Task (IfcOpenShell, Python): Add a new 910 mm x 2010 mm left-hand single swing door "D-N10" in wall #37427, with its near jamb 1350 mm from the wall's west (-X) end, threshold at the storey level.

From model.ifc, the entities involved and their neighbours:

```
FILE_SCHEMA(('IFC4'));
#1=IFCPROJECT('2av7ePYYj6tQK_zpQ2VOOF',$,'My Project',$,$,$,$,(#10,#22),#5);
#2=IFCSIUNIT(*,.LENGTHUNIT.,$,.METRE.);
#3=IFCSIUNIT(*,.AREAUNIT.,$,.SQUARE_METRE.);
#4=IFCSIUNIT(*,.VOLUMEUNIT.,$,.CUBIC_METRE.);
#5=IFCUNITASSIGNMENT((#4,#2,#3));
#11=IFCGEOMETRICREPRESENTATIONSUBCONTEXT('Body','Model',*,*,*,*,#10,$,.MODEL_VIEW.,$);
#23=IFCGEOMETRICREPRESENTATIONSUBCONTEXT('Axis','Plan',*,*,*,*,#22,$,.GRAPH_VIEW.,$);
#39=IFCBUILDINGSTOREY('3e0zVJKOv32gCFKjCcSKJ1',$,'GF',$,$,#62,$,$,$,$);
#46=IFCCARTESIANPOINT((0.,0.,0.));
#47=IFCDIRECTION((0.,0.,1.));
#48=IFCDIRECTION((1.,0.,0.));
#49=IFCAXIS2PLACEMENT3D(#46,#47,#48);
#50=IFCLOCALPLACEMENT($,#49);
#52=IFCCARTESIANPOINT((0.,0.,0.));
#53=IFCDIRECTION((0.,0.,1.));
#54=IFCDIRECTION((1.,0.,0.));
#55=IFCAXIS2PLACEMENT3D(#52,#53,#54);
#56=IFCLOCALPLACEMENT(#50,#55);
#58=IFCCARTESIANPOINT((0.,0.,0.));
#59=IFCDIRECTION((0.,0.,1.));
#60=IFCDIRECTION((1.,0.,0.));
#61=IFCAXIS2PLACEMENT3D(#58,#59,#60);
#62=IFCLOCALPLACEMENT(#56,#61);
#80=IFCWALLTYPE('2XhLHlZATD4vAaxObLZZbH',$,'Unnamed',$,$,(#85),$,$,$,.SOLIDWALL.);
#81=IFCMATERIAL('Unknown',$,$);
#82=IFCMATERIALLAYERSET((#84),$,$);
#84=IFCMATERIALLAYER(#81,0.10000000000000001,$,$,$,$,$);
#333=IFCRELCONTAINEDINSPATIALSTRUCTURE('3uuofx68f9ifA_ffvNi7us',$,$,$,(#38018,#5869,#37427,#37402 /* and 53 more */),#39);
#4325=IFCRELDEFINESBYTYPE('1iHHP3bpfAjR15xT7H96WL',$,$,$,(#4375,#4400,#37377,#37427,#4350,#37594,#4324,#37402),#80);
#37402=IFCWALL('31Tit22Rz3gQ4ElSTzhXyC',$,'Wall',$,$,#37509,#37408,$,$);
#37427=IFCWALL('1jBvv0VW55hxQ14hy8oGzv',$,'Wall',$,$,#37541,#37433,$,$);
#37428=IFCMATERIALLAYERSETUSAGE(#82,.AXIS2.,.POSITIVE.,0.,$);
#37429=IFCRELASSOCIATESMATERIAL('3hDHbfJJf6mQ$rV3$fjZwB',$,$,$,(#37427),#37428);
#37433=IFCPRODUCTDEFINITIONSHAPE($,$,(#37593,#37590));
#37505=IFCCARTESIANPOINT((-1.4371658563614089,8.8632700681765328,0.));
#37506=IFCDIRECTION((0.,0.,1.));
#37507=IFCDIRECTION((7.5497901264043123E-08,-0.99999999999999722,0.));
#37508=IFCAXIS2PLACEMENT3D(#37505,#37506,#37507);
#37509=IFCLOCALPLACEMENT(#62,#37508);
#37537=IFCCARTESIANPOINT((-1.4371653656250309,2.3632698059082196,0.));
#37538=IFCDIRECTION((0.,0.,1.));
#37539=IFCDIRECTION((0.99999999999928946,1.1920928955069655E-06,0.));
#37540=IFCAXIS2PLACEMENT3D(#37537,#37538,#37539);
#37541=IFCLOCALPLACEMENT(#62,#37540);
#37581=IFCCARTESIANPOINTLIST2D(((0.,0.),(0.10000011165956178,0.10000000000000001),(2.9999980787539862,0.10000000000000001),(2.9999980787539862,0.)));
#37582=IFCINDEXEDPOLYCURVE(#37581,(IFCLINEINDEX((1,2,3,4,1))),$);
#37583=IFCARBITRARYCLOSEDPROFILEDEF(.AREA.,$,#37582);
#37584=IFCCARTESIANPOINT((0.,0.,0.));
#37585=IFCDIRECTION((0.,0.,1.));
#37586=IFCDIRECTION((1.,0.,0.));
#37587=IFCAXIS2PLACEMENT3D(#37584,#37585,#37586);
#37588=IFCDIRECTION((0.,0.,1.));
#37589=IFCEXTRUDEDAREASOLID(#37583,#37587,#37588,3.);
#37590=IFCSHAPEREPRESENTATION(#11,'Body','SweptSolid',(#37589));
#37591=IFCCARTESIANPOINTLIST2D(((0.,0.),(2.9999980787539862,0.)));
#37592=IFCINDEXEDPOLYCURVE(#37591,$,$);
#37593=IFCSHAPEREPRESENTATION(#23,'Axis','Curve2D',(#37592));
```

```python
import numpy as np
import ifcopenshell
import ifcopenshell.api.feature
import ifcopenshell.api.geometry
import ifcopenshell.api.root
import ifcopenshell.api.spatial
import ifcopenshell.geom
import ifcopenshell.util.element
import ifcopenshell.util.placement
import ifcopenshell.util.representation
import ifcopenshell.util.shape
import ifcopenshell.util.unit

model = ifcopenshell.open("model.ifc")
unit_scale = ifcopenshell.util.unit.calculate_unit_scale(model)
settings = ifcopenshell.geom.settings()


def volume(element):
    """Net volume in cubic metres, openings subtracted."""
    shape = ifcopenshell.geom.create_shape(settings, element)
    return ifcopenshell.util.shape.get_volume(shape.geometry)


wall = model.by_guid("1jBvv0VW55hxQ14hy8oGzv")
storey = ifcopenshell.util.element.get_container(wall, ifc_class="IfcBuildingStorey")
context = ifcopenshell.util.representation.get_context(model, "Model", "Body", "MODEL_VIEW")
before = volume(wall)

width, height, from_end, sill = 0.91, 2.01, 1.35, 0.0  # metres

# The wall runs along its own X axis, and the end named is its -X end.
wall_shape = ifcopenshell.geom.create_shape(settings, wall)
x, y, z = ifcopenshell.util.shape.get_vertices(wall_shape.geometry).T
start = x.min() + from_end
face, thickness = float(y.min()), float(y.max() - y.min())
wall_matrix = ifcopenshell.util.placement.get_local_placement(wall.ObjectPlacement)
level = ifcopenshell.util.placement.get_local_placement(storey.ObjectPlacement)[2, 3]


def in_wall(x, y):
    """Placement at x, y metres in the wall's axes, at sill height."""
    matrix = wall_matrix.copy()
    matrix[:, 3] = wall_matrix @ np.array([x / unit_scale, y / unit_scale, 0.0, 1.0])
    matrix[2, 3] = level + sill / unit_scale
    return matrix


# Opening: a box that overshoots both wall faces by 50 mm.
opening = ifcopenshell.api.root.create_entity(model, ifc_class="IfcOpeningElement", predefined_type="OPENING")
box = ifcopenshell.api.geometry.add_wall_representation(
    model, context=context, length=width, height=height, thickness=thickness + 0.1
)
ifcopenshell.api.geometry.assign_representation(model, product=opening, representation=box)
ifcopenshell.api.geometry.edit_object_placement(model, product=opening, matrix=in_wall(start, face - 0.05), is_si=False)
ifcopenshell.api.feature.add_feature(model, feature=opening, element=wall)

door = ifcopenshell.api.root.create_entity(model, ifc_class="IfcDoor", name="D-N10", predefined_type="DOOR")
door.OverallWidth, door.OverallHeight = width / unit_scale, height / unit_scale
door.OperationType = "SINGLE_SWING_LEFT"
body = ifcopenshell.api.geometry.add_door_representation(
    model,
    context=context,
    overall_width=door.OverallWidth,
    overall_height=door.OverallHeight,
    operation_type="SINGLE_SWING_LEFT",
    lining_properties={"LiningDepth": thickness / unit_scale, "ThresholdDepth": thickness / unit_scale},
)
ifcopenshell.api.geometry.assign_representation(model, product=door, representation=body)
ifcopenshell.api.spatial.assign_container(model, products=[door], relating_structure=storey)
ifcopenshell.api.feature.add_filling(model, opening=opening, element=door)

# The lining spans the wall, so the door starts at the wall face.
ifcopenshell.api.geometry.edit_object_placement(model, product=door, matrix=in_wall(start, face), is_si=False)

after = volume(wall)

print(f"wall volume {before:.3f} -> {after:.3f} m3")

model.write("model_edited.ifc")
```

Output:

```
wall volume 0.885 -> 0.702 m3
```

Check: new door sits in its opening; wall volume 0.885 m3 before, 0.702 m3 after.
